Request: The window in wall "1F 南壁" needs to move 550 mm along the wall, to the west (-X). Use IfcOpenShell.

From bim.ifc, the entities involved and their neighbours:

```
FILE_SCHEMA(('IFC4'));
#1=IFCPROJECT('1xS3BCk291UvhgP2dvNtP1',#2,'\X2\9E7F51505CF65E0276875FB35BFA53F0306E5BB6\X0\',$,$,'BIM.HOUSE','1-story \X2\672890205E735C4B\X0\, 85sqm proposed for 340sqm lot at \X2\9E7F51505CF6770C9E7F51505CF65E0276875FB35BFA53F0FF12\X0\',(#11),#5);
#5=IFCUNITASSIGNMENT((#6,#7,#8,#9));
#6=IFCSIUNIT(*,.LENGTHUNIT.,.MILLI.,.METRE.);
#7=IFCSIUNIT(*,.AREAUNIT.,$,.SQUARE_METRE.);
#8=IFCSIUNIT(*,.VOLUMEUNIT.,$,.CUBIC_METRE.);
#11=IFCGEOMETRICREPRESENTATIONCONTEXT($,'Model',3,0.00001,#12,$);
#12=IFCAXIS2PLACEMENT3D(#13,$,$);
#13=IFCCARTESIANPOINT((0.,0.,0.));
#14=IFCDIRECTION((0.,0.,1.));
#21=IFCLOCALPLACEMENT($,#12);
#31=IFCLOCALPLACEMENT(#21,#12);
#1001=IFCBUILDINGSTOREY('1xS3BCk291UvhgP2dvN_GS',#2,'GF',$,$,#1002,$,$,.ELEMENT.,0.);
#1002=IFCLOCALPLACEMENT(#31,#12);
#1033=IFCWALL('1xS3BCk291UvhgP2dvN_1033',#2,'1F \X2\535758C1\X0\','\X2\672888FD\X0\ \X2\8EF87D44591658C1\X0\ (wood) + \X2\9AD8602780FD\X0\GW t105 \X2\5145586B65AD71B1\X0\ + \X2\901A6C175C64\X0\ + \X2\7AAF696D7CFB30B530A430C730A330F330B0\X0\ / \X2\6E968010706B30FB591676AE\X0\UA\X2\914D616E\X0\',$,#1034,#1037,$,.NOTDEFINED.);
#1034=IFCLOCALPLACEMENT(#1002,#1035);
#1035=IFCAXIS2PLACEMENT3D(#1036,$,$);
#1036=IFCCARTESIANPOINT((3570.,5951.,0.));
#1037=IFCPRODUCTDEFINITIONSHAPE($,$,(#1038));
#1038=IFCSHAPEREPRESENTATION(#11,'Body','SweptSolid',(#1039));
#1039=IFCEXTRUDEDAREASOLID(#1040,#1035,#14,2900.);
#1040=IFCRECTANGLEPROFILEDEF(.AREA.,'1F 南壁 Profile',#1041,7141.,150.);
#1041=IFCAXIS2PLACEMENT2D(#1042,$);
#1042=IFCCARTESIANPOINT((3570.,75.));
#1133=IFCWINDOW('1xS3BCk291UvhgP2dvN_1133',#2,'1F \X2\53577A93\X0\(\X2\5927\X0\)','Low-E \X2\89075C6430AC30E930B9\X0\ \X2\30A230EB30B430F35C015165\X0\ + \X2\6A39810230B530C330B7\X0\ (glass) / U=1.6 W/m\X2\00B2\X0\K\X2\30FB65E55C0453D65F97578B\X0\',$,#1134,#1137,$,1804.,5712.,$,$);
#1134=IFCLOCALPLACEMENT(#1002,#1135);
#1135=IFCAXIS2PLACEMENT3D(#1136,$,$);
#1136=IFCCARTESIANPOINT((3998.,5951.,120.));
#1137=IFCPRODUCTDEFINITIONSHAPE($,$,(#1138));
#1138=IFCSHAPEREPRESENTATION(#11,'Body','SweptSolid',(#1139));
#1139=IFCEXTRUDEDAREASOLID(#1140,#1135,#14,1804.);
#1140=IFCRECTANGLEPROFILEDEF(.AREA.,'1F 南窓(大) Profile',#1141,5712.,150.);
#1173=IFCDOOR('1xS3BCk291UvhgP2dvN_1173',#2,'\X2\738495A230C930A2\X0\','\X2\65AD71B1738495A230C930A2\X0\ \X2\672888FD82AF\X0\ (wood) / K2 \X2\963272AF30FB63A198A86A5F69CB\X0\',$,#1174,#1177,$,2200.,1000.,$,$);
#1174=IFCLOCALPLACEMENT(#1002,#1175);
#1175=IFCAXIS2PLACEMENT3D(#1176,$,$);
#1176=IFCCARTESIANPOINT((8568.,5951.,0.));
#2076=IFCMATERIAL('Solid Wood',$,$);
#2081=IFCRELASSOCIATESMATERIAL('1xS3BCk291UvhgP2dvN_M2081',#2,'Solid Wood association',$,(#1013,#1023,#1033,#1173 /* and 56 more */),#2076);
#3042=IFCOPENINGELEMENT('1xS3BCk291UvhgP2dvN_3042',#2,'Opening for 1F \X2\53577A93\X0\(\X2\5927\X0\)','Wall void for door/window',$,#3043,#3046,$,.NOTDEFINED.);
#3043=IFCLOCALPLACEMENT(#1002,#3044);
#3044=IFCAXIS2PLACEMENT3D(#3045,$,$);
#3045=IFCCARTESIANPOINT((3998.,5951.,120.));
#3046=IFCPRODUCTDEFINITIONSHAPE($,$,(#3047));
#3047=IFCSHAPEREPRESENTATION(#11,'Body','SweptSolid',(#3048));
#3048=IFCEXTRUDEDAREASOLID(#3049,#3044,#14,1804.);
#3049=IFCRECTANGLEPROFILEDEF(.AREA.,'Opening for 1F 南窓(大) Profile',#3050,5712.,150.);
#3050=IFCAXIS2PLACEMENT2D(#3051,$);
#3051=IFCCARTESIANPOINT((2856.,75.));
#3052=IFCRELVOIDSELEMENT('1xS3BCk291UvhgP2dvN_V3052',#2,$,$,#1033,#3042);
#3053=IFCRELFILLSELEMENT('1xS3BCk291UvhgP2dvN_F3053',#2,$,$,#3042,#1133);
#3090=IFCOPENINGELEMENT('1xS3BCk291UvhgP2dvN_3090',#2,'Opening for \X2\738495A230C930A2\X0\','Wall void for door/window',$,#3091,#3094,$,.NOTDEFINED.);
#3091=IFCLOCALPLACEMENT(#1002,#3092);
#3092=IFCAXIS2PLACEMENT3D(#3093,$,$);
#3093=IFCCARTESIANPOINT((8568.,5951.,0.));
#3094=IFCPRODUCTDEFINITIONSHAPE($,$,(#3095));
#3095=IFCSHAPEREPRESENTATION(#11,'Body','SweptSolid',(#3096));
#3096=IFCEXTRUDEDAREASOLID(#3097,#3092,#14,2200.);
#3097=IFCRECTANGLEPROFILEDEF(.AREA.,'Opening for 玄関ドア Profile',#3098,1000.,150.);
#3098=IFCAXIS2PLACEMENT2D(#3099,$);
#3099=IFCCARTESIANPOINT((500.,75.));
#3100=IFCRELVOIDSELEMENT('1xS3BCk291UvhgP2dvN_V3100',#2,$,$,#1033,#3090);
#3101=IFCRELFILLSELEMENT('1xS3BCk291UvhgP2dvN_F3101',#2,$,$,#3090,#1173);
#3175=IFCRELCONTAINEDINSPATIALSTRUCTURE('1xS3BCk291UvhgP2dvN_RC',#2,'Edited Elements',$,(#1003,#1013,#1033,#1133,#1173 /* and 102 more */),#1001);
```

```python
import ifcopenshell
import ifcopenshell.api.geometry
import ifcopenshell.util.placement
import ifcopenshell.util.unit

model = ifcopenshell.open("bim.ifc")
unit_scale = ifcopenshell.util.unit.calculate_unit_scale(model)

window = model.by_guid("1xS3BCk291UvhgP2dvN_1133")
opening = window.FillsVoids[0].RelatingOpeningElement
wall = opening.VoidsElements[0].RelatingBuildingElement

wall_matrix = ifcopenshell.util.placement.get_local_placement(wall.ObjectPlacement)
shift = wall_matrix[:3, 0] * -0.55 / unit_scale
before = ifcopenshell.util.placement.get_local_placement(window.ObjectPlacement)[:3, 3].copy()

# The window is not placed relative to its opening, so move both.
for product in (opening, window):
    matrix = ifcopenshell.util.placement.get_local_placement(product.ObjectPlacement)
    matrix[:3, 3] += shift
    ifcopenshell.api.geometry.edit_object_placement(model, product=product, matrix=matrix, is_si=False)

after = ifcopenshell.util.placement.get_local_placement(window.ObjectPlacement)[:3, 3]
print("window moved by", (after - before).round(3) + 0.0)

model.write("bim-out.ifc")
```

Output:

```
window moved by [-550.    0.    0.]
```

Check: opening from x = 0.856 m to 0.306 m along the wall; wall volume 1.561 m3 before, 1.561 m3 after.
